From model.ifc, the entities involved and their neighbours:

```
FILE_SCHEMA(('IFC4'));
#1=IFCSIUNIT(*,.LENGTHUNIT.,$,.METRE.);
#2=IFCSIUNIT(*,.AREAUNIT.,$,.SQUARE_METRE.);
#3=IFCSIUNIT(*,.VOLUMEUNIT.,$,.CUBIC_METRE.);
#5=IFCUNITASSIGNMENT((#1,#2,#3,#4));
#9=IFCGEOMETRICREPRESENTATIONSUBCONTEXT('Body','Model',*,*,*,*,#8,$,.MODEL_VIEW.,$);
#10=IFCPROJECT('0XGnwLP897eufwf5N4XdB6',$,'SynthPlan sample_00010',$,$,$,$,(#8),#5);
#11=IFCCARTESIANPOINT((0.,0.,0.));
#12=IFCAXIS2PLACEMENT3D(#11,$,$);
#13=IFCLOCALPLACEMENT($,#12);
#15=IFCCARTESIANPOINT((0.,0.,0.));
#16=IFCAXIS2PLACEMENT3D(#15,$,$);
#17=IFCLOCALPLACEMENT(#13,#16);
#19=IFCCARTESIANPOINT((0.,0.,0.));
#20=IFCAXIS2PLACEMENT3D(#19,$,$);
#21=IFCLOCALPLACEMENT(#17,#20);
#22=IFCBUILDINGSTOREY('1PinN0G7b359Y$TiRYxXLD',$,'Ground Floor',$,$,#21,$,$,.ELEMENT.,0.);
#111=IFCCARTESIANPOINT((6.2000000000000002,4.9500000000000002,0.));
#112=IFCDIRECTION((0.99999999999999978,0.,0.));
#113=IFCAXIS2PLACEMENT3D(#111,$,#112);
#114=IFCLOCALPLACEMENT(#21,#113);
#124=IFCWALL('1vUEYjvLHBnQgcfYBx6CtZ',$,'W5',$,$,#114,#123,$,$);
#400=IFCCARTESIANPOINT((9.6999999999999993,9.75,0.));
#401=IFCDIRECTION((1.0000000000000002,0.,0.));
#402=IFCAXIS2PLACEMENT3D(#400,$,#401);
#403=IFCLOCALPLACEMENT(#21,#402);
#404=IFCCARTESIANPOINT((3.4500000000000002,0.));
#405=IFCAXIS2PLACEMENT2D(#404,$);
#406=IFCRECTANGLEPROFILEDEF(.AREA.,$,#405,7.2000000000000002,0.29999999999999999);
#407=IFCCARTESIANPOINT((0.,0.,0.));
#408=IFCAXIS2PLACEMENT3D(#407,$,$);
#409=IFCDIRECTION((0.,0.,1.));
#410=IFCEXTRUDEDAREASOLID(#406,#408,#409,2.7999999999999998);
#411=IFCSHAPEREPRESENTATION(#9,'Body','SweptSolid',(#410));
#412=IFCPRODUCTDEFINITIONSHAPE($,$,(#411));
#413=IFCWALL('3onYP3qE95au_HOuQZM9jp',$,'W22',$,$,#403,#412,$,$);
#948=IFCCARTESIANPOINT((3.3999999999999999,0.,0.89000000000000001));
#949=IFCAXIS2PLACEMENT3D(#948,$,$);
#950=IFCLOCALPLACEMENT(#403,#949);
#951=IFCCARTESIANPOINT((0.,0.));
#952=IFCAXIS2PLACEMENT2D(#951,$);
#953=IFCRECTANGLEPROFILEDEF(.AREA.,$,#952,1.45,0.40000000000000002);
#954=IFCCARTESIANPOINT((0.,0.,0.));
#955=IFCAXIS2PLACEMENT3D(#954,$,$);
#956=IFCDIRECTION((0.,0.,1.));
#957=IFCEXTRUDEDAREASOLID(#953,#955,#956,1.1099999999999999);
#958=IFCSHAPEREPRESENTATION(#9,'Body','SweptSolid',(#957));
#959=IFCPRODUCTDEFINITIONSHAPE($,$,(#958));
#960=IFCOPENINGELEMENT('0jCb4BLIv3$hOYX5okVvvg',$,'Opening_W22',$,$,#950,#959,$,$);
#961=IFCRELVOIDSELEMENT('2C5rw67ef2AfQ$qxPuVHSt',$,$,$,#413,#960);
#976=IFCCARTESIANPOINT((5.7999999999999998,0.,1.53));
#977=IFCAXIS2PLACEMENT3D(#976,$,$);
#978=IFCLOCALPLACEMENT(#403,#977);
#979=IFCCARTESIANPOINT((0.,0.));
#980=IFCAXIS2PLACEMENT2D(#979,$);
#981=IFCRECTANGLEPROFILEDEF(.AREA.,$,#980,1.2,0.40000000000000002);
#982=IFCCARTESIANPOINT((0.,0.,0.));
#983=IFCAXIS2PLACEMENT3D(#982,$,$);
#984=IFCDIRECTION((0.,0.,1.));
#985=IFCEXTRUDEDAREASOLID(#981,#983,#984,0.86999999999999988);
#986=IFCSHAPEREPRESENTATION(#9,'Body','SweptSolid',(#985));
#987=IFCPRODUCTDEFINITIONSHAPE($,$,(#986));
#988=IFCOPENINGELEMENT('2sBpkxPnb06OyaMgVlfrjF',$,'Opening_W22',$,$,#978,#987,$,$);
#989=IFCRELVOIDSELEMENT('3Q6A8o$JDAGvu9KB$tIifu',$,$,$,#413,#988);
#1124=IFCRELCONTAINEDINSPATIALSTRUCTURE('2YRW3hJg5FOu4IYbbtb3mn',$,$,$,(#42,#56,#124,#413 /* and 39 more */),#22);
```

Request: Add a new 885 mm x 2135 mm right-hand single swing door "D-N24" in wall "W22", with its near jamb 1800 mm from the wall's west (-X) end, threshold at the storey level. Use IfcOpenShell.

```python
import numpy as np
import ifcopenshell
import ifcopenshell.api.feature
import ifcopenshell.api.geometry
import ifcopenshell.api.root
import ifcopenshell.api.spatial
import ifcopenshell.geom
import ifcopenshell.util.element
import ifcopenshell.util.placement
import ifcopenshell.util.representation
import ifcopenshell.util.shape
import ifcopenshell.util.unit

model = ifcopenshell.open("model.ifc")
unit_scale = ifcopenshell.util.unit.calculate_unit_scale(model)
settings = ifcopenshell.geom.settings()


def volume(element):
    """Net volume in cubic metres, openings subtracted."""
    shape = ifcopenshell.geom.create_shape(settings, element)
    return ifcopenshell.util.shape.get_volume(shape.geometry)


wall = model.by_guid("3onYP3qE95au_HOuQZM9jp")
storey = ifcopenshell.util.element.get_container(wall, ifc_class="IfcBuildingStorey")
context = ifcopenshell.util.representation.get_context(model, "Model", "Body", "MODEL_VIEW")
before = volume(wall)

width, height, from_end, sill = 0.885, 2.135, 1.8, 0.0  # metres

# The wall runs along its own X axis, and the end named is its -X end.
wall_shape = ifcopenshell.geom.create_shape(settings, wall)
x, y, z = ifcopenshell.util.shape.get_vertices(wall_shape.geometry).T
start = x.min() + from_end
face, thickness = float(y.min()), float(y.max() - y.min())
wall_matrix = ifcopenshell.util.placement.get_local_placement(wall.ObjectPlacement)
level = ifcopenshell.util.placement.get_local_placement(storey.ObjectPlacement)[2, 3]


def in_wall(x, y):
    """Placement at x, y metres in the wall's axes, at sill height."""
    matrix = wall_matrix.copy()
    matrix[:, 3] = wall_matrix @ np.array([x / unit_scale, y / unit_scale, 0.0, 1.0])
    matrix[2, 3] = level + sill / unit_scale
    return matrix


# Opening: a box that overshoots both wall faces by 50 mm.
opening = ifcopenshell.api.root.create_entity(model, ifc_class="IfcOpeningElement", predefined_type="OPENING")
box = ifcopenshell.api.geometry.add_wall_representation(
    model, context=context, length=width, height=height, thickness=thickness + 0.1
)
ifcopenshell.api.geometry.assign_representation(model, product=opening, representation=box)
ifcopenshell.api.geometry.edit_object_placement(model, product=opening, matrix=in_wall(start, face - 0.05), is_si=False)
ifcopenshell.api.feature.add_feature(model, feature=opening, element=wall)

door = ifcopenshell.api.root.create_entity(model, ifc_class="IfcDoor", name="D-N24", predefined_type="DOOR")
door.OverallWidth, door.OverallHeight = width / unit_scale, height / unit_scale
door.OperationType = "SINGLE_SWING_RIGHT"
body = ifcopenshell.api.geometry.add_door_representation(
    model,
    context=context,
    overall_width=door.OverallWidth,
    overall_height=door.OverallHeight,
    operation_type="SINGLE_SWING_RIGHT",
    lining_properties={"LiningDepth": thickness / unit_scale, "ThresholdDepth": thickness / unit_scale},
)
ifcopenshell.api.geometry.assign_representation(model, product=door, representation=body)
ifcopenshell.api.spatial.assign_container(model, products=[door], relating_structure=storey)
ifcopenshell.api.feature.add_filling(model, opening=opening, element=door)

# The lining spans the wall, so the door starts at the wall face.
ifcopenshell.api.geometry.edit_object_placement(model, product=door, matrix=in_wall(start, face), is_si=False)

after = volume(wall)

print(f"wall volume {before:.3f} -> {after:.3f} m3")

model.write("model_edited.ifc")
```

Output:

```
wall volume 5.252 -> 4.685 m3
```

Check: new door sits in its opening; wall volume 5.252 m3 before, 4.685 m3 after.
